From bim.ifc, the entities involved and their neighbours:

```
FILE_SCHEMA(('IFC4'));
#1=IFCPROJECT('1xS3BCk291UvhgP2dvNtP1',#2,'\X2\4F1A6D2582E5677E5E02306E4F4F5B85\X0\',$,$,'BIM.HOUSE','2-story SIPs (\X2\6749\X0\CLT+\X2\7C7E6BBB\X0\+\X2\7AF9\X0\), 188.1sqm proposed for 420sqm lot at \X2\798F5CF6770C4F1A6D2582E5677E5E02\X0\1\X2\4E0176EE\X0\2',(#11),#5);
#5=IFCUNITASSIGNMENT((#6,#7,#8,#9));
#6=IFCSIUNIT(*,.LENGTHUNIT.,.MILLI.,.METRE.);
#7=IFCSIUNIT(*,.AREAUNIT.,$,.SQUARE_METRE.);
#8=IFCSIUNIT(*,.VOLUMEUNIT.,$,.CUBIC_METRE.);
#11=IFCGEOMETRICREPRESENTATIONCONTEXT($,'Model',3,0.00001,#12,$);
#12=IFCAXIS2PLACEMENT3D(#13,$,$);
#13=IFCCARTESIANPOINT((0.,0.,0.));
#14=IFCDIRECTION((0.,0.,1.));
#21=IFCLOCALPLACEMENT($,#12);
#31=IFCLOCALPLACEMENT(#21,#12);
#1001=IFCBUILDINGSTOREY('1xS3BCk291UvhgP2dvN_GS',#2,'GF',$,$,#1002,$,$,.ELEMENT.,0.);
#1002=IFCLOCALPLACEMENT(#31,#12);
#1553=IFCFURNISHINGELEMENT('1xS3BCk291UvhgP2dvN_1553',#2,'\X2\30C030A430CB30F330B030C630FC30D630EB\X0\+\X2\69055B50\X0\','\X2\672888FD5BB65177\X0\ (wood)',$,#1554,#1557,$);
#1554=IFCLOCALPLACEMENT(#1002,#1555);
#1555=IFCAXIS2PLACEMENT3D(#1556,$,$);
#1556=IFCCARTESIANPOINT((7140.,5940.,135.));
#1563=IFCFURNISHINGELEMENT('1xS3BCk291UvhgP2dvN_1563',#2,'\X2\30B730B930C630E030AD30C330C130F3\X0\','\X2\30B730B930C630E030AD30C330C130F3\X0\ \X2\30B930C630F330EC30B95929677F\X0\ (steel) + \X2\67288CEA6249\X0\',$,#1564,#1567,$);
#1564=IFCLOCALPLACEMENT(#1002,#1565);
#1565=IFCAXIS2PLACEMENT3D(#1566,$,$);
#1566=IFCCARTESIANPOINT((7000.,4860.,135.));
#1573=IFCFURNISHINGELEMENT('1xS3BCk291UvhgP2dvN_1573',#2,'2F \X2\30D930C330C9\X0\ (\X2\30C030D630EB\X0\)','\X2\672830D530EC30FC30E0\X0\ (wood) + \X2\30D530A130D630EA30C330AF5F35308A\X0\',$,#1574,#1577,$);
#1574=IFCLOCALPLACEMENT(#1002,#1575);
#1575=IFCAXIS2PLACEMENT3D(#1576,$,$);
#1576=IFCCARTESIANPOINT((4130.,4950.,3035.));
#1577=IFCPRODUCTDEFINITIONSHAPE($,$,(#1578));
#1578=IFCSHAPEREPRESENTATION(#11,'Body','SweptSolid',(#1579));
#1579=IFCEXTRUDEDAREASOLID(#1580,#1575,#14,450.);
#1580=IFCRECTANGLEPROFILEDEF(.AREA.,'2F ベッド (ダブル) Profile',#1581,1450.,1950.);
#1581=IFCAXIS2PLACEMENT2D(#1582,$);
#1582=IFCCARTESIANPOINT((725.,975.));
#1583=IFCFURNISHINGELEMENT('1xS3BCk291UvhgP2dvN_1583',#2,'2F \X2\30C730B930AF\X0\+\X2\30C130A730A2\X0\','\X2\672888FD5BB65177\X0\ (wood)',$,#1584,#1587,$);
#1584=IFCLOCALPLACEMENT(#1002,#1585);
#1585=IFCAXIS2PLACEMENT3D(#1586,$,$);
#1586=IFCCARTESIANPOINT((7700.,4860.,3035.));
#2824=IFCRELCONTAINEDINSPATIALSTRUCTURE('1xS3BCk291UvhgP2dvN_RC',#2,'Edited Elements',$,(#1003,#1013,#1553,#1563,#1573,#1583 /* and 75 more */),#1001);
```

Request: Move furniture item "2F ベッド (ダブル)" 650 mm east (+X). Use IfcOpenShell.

```python
import ifcopenshell
import ifcopenshell.api.geometry
import ifcopenshell.util.placement

model = ifcopenshell.open("bim.ifc")

item = model.by_id(1573)
matrix = ifcopenshell.util.placement.get_local_placement(item.ObjectPlacement)
matrix[0, 3] += 650.0
ifcopenshell.api.geometry.edit_object_placement(model, product=item, matrix=matrix, is_si=False)

print(ifcopenshell.util.placement.get_local_placement(item.ObjectPlacement).round(3) + 0.0)

model.write("bim-out.ifc")
```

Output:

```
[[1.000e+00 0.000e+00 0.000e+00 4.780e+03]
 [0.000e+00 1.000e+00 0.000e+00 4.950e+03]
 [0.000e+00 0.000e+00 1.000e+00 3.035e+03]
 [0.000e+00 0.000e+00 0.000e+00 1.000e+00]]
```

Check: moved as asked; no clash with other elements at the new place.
